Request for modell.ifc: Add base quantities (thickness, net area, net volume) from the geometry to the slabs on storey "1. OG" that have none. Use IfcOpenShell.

First a look at what the model holds.

```python
import ifcopenshell
import ifcopenshell.util.element
import ifcopenshell.util.unit

model = ifcopenshell.open("modell.ifc")
print(model.schema)
for unit_type in ("LENGTHUNIT", "AREAUNIT", "VOLUMEUNIT"):
    print(unit_type, ifcopenshell.util.unit.calculate_unit_scale(model, unit_type))
storey = next(s for s in model.by_type("IfcBuildingStorey") if s.Name == "1. OG")
slabs = [e for e in ifcopenshell.util.element.get_decomposition(storey) if e.is_a("IfcSlab")]
for e in sorted(slabs, key=lambda e: e.id()):
    print(e.id(), e.is_a(), e.Name, list(ifcopenshell.util.element.get_psets(e, qtos_only=True)), sep=" | ")
```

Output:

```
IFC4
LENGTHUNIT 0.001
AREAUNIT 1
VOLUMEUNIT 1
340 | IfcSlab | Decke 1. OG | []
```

```python
import ifcopenshell
import ifcopenshell.api.pset
import ifcopenshell.geom
import ifcopenshell.util.element
import ifcopenshell.util.shape
import ifcopenshell.util.unit

model = ifcopenshell.open("modell.ifc")
unit_scale = ifcopenshell.util.unit.calculate_unit_scale(model)
area_scale = ifcopenshell.util.unit.calculate_unit_scale(model, "AREAUNIT")
volume_scale = ifcopenshell.util.unit.calculate_unit_scale(model, "VOLUMEUNIT")
settings = ifcopenshell.geom.settings()

storey = next(s for s in model.by_type("IfcBuildingStorey") if s.Name == "1. OG")
slabs = [e for e in ifcopenshell.util.element.get_decomposition(storey) if e.is_a("IfcSlab")]

for e in sorted(slabs, key=lambda e: e.id()):
    if ifcopenshell.util.element.get_psets(e, qtos_only=True, should_inherit=False):
        continue
    # Geometry comes back in metres, in the element's own axes.
    shape = ifcopenshell.geom.create_shape(settings, e)
    values = {
        "Width": ifcopenshell.util.shape.get_z(shape.geometry) / unit_scale,
        "NetArea": ifcopenshell.util.shape.get_footprint_area(shape.geometry) / area_scale,
        "NetVolume": ifcopenshell.util.shape.get_volume(shape.geometry) / volume_scale,
    }
    qto = ifcopenshell.api.pset.add_qto(model, product=e, name="Qto_SlabBaseQuantities")
    ifcopenshell.api.pset.edit_qto(model, qto=qto, properties=values)
    print(e.id(), {k: round(v, 3) for k, v in values.items()})

model.write("modell-out.ifc")
```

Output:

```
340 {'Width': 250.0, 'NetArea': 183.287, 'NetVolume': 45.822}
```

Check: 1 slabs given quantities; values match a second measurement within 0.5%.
